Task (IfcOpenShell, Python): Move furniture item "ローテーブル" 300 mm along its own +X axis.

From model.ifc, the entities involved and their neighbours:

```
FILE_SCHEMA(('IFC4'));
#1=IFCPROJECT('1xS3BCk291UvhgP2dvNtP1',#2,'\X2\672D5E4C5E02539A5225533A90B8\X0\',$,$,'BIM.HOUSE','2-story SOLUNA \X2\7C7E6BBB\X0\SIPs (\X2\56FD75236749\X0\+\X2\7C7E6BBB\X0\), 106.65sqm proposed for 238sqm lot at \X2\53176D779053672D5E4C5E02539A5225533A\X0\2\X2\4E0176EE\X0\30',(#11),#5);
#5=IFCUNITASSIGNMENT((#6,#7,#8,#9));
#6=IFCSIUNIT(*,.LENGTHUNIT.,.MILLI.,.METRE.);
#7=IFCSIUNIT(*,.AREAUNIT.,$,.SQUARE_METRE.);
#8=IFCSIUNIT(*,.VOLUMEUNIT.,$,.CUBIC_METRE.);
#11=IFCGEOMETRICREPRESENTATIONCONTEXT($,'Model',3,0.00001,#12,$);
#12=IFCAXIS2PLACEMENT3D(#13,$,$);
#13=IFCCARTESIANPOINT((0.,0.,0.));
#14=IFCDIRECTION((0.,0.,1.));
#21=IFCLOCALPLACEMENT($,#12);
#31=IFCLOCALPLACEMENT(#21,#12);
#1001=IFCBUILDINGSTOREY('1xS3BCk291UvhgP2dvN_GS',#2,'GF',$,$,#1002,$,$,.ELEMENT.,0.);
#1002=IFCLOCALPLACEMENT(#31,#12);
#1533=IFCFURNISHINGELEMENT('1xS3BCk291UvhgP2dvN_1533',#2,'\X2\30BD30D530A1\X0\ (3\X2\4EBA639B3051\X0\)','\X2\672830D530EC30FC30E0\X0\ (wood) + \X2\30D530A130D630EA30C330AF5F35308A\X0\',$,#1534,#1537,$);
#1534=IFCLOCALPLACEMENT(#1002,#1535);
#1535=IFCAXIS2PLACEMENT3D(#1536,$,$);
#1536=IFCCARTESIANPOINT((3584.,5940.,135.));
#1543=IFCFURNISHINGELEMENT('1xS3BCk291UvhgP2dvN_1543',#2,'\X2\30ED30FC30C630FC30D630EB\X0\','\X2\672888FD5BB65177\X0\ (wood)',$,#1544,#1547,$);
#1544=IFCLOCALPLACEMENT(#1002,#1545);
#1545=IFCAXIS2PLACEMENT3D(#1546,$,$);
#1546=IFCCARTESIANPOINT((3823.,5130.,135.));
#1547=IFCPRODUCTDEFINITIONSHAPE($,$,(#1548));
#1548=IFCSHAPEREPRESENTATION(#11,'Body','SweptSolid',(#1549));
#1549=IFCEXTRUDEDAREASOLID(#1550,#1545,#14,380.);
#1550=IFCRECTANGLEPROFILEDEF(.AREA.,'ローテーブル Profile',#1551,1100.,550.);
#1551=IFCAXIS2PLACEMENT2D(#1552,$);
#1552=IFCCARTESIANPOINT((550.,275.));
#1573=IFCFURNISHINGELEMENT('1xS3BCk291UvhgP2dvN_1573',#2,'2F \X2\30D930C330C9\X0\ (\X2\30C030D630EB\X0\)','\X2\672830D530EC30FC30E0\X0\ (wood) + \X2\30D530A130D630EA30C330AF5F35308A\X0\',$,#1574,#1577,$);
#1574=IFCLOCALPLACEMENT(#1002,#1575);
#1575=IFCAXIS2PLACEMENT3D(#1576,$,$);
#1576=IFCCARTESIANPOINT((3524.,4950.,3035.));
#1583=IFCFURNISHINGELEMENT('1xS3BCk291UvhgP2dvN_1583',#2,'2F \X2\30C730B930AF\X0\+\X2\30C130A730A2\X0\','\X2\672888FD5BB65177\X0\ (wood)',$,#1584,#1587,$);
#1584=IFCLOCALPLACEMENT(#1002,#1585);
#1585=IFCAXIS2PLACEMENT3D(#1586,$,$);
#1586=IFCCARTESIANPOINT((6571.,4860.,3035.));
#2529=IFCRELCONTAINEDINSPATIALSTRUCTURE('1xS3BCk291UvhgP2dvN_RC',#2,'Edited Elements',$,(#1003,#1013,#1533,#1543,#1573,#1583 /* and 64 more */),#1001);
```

```python
import ifcopenshell
import ifcopenshell.api.geometry
import ifcopenshell.util.placement

model = ifcopenshell.open("model.ifc")

item = model.by_guid("1xS3BCk291UvhgP2dvN_1543")
matrix = ifcopenshell.util.placement.get_local_placement(item.ObjectPlacement)
matrix[:3, 3] += matrix[:3, 0] * 300.0
ifcopenshell.api.geometry.edit_object_placement(model, product=item, matrix=matrix, is_si=False)

print(ifcopenshell.util.placement.get_local_placement(item.ObjectPlacement).round(3) + 0.0)

model.write("model_rev.ifc")
```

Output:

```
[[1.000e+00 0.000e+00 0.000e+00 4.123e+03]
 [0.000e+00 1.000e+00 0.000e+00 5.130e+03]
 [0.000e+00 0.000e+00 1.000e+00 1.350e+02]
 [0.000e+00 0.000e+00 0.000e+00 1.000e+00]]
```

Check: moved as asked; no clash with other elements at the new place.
